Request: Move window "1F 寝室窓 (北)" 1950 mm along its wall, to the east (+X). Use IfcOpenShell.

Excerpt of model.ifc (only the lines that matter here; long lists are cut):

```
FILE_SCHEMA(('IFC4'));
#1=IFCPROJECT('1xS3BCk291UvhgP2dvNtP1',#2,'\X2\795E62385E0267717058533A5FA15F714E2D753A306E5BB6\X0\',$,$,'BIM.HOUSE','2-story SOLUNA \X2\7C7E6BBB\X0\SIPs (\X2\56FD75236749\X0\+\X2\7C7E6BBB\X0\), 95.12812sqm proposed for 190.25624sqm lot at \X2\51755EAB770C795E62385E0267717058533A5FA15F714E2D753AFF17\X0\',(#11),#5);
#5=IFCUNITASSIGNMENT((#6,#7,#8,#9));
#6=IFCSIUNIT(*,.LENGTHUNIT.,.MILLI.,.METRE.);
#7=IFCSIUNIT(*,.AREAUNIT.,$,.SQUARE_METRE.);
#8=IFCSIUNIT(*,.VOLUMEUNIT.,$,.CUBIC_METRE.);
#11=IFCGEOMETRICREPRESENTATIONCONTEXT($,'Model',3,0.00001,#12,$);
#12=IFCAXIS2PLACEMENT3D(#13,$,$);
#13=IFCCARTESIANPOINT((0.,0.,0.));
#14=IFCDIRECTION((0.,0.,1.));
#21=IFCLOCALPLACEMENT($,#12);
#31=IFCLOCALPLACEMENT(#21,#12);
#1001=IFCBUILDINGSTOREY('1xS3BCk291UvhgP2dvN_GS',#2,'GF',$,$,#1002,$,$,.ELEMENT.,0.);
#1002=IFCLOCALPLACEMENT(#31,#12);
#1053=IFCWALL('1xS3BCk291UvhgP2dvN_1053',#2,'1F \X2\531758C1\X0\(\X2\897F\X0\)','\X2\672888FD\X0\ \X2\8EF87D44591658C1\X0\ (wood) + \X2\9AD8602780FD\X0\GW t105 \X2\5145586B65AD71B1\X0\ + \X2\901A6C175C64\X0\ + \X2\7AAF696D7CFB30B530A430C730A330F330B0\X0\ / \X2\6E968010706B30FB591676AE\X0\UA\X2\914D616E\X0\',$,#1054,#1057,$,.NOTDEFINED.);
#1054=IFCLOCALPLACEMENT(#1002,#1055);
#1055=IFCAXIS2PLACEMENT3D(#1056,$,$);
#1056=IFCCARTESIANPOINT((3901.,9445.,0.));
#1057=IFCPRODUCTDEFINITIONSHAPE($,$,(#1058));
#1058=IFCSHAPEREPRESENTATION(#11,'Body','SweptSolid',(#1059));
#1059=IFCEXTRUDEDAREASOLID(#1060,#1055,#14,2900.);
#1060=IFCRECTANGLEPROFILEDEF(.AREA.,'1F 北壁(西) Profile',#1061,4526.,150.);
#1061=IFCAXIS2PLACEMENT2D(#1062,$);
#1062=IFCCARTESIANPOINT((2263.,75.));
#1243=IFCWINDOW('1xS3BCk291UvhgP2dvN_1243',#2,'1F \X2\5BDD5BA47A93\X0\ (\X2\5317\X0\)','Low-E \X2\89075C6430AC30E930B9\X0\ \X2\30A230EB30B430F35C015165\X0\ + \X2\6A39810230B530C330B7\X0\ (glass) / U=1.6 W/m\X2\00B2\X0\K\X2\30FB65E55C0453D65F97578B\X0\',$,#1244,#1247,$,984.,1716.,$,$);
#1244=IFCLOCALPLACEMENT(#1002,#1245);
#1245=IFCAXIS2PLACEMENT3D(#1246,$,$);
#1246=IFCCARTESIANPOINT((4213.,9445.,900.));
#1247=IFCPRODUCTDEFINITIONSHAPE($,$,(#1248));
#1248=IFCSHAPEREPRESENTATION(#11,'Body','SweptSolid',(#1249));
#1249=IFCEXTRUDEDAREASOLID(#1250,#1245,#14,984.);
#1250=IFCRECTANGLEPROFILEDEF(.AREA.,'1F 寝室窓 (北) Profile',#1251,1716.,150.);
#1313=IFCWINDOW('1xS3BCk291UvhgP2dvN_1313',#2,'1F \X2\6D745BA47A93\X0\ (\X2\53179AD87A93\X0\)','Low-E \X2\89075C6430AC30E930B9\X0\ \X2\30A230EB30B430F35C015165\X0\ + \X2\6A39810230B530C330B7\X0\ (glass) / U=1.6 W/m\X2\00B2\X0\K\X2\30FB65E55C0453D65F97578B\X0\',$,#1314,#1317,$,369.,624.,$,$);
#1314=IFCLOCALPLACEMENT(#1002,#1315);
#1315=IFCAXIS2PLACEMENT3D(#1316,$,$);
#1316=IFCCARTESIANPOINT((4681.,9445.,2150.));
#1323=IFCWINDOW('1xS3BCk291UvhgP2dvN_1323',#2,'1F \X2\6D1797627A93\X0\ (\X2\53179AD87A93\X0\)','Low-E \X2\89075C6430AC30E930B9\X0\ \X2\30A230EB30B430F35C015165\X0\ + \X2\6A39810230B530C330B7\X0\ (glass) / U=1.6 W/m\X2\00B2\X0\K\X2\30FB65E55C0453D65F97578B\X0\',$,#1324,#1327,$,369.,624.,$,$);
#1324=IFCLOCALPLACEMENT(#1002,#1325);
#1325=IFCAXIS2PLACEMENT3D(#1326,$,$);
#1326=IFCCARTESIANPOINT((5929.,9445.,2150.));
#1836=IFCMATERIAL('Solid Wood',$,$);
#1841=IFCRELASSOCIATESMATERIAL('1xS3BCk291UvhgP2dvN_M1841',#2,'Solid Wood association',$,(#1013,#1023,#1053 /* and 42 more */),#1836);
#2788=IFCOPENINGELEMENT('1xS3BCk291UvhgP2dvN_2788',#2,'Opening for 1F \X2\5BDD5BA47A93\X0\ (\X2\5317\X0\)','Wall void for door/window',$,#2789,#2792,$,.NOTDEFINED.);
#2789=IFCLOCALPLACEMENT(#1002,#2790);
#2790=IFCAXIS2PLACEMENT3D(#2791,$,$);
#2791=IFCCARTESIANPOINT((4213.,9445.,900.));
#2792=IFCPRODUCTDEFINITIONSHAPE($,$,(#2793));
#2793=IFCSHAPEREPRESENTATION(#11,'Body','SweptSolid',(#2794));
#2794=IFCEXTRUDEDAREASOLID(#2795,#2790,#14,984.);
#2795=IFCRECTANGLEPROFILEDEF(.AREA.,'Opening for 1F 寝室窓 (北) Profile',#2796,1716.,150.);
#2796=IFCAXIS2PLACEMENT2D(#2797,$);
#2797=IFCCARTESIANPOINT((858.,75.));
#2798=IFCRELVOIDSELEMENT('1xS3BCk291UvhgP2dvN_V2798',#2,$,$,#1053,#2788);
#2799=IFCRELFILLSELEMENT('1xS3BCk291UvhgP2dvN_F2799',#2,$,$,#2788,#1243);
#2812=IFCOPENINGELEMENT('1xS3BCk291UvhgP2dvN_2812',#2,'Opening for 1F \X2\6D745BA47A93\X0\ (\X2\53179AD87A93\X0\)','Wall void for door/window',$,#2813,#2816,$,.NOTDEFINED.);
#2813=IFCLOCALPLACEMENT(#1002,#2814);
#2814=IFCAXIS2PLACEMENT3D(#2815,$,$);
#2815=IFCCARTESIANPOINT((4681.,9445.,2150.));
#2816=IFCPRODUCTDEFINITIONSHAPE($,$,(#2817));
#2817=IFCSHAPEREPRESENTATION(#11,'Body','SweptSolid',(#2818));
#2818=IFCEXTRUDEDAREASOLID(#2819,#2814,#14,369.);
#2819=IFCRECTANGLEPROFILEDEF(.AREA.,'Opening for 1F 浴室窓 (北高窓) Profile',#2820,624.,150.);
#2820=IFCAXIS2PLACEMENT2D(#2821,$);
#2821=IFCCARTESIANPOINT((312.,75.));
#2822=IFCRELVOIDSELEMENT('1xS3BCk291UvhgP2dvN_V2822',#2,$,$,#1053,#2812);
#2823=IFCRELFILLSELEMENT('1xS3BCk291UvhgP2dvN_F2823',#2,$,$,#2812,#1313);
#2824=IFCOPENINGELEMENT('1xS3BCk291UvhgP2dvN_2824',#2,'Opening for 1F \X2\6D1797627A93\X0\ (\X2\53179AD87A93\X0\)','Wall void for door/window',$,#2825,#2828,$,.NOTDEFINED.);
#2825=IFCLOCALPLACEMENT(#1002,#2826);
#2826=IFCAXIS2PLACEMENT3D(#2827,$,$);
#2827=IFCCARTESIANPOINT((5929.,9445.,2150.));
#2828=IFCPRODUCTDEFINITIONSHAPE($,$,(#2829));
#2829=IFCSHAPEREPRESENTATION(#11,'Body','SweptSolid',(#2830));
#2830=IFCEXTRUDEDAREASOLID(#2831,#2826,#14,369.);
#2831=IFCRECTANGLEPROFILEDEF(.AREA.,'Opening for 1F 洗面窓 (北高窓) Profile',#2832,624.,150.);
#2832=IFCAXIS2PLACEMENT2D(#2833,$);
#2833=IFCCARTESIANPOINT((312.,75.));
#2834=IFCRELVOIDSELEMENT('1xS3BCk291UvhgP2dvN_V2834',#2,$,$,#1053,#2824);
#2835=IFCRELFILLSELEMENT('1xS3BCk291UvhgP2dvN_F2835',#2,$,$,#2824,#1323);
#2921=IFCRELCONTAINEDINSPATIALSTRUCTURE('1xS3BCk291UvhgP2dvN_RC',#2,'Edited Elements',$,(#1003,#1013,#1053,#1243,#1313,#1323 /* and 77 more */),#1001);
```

```python
import ifcopenshell
import ifcopenshell.api.geometry
import ifcopenshell.util.placement
import ifcopenshell.util.unit

model = ifcopenshell.open("model.ifc")
unit_scale = ifcopenshell.util.unit.calculate_unit_scale(model)

window = model.by_guid("1xS3BCk291UvhgP2dvN_1243")
opening = window.FillsVoids[0].RelatingOpeningElement
wall = opening.VoidsElements[0].RelatingBuildingElement

wall_matrix = ifcopenshell.util.placement.get_local_placement(wall.ObjectPlacement)
shift = wall_matrix[:3, 0] * 1.95 / unit_scale
before = ifcopenshell.util.placement.get_local_placement(window.ObjectPlacement)[:3, 3].copy()

# The window is not placed relative to its opening, so move both.
for product in (opening, window):
    matrix = ifcopenshell.util.placement.get_local_placement(product.ObjectPlacement)
    matrix[:3, 3] += shift
    ifcopenshell.api.geometry.edit_object_placement(model, product=product, matrix=matrix, is_si=False)

after = ifcopenshell.util.placement.get_local_placement(window.ObjectPlacement)[:3, 3]
print("window moved by", (after - before).round(3) + 0.0)

model.write("model_rev.ifc")
```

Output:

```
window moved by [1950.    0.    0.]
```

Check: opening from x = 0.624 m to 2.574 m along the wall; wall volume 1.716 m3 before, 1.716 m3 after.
